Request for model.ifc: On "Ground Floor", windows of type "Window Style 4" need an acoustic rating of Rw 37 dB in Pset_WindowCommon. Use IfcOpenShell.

First a look at what the model holds.

```python
import ifcopenshell
import ifcopenshell.util.element

model = ifcopenshell.open("model.ifc")
print(model.schema)
storey = next(s for s in model.by_type("IfcBuildingStorey") if s.Name == "Ground Floor")
windows = [e for e in ifcopenshell.util.element.get_decomposition(storey) if e.is_a("IfcWindow")]
seen = {}
for e in windows:
    element_type = ifcopenshell.util.element.get_type(e)
    key = (element_type.Name if element_type != e and element_type else None, ifcopenshell.util.element.get_pset(e, "Pset_WindowCommon", "AcousticRating"))
    seen[key] = seen.get(key, 0) + 1
for (name, value), count in sorted(seen.items(), key=str):
    print(count, "x", name, "|", value)
```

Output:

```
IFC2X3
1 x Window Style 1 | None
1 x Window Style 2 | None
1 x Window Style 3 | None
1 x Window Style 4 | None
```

```python
import ifcopenshell
import ifcopenshell.api.pset
import ifcopenshell.util.element

model = ifcopenshell.open("model.ifc")

storey = next(s for s in model.by_type("IfcBuildingStorey") if s.Name == "Ground Floor")
windows = [e for e in ifcopenshell.util.element.get_decomposition(storey) if e.is_a("IfcWindow")]

count = 0
for e in windows:
    element_type = ifcopenshell.util.element.get_type(e)
    if element_type in (None, e) or element_type.Name != "Window Style 4":
        continue
    # add_pset returns the element's existing set when there is one.
    pset = ifcopenshell.api.pset.add_pset(model, product=e, name="Pset_WindowCommon")
    ifcopenshell.api.pset.edit_pset(model, pset=pset, properties={"AcousticRating": "Rw 37 dB"})
    count += 1

print(count, "windows updated")

model.write("model_updated.ifc")
```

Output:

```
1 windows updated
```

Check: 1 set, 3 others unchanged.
